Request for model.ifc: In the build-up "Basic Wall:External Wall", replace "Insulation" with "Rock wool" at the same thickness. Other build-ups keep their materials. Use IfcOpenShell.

First a look at what the model holds.

```python
import ifcopenshell
import ifcopenshell.util.element

model = ifcopenshell.open("model.ifc")
print(model.schema)
for layer_set in model.by_type("IfcMaterialLayerSet"):
    if layer_set.LayerSetName == "Basic Wall:External Wall":
        for layer in layer_set.MaterialLayers:
            print(layer.id(), layer.Material and layer.Material.Name, layer.LayerThickness, sep=" | ")
        print(len(ifcopenshell.util.element.get_elements_by_material(model, layer_set)), "elements and types use it")
print(sorted(m.Name for m in model.by_type("IfcMaterial") if m.Name)[:60])
```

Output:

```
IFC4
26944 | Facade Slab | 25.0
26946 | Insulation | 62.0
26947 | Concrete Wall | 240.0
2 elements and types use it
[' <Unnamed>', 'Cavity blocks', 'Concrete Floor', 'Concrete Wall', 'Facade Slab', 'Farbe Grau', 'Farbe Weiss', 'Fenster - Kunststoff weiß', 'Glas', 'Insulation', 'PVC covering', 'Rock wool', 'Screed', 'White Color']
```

```python
import ifcopenshell
import ifcopenshell.api.material

model = ifcopenshell.open("model.ifc")

layer_set = next(s for s in model.by_type("IfcMaterialLayerSet") if s.LayerSetName == "Basic Wall:External Wall")
layer = next(l for l in layer_set.MaterialLayers if l.Material and l.Material.Name == "Insulation")
material = next(m for m in model.by_type("IfcMaterial") if m.Name == "Rock wool")

# Point this one layer at the other material; renaming the old one would change it everywhere.
ifcopenshell.api.material.edit_layer(model, layer=layer, attributes={}, material=material)

print([l.Material.Name if l.Material else None for l in layer_set.MaterialLayers])

model.write("model_v2.ifc")
```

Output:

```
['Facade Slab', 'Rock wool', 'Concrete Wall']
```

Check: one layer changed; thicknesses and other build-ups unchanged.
